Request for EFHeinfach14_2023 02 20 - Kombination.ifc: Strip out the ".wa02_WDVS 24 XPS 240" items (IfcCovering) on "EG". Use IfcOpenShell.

First a look at what the model holds.

```python
import ifcopenshell
import ifcopenshell.util.element

model = ifcopenshell.open("EFHeinfach14_2023 02 20 - Kombination.ifc")
print(model.schema)
storey = next(s for s in model.by_type("IfcBuildingStorey") if s.Name == "EG")
coverings = [e for e in ifcopenshell.util.element.get_decomposition(storey) if e.is_a("IfcCovering")]
seen = {}
for e in coverings:
    element_type = ifcopenshell.util.element.get_type(e)
    name = element_type.Name if element_type not in (None, e) else None
    seen[name] = seen.get(name, 0) + 1
for name, count in sorted(seen.items(), key=str):
    print(count, "x", name)
```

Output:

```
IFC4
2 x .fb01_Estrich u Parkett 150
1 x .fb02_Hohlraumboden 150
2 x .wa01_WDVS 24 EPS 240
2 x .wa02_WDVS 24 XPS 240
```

```python
import ifcopenshell
import ifcopenshell.api.root
import ifcopenshell.util.element

model = ifcopenshell.open("EFHeinfach14_2023 02 20 - Kombination.ifc")

storey = next(s for s in model.by_type("IfcBuildingStorey") if s.Name == "EG")
coverings = [e for e in ifcopenshell.util.element.get_decomposition(storey) if e.is_a("IfcCovering")]
targets = [e for e in coverings if (t := ifcopenshell.util.element.get_type(e)) not in (None, e) and t.Name == ".wa02_WDVS 24 XPS 240"]

for e in targets:
    ifcopenshell.api.root.remove_product(model, product=e)
print(len(targets), "removed")

model.write("EFHeinfach14_2023 02 20 - Kombination-out.ifc")
```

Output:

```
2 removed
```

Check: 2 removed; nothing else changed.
